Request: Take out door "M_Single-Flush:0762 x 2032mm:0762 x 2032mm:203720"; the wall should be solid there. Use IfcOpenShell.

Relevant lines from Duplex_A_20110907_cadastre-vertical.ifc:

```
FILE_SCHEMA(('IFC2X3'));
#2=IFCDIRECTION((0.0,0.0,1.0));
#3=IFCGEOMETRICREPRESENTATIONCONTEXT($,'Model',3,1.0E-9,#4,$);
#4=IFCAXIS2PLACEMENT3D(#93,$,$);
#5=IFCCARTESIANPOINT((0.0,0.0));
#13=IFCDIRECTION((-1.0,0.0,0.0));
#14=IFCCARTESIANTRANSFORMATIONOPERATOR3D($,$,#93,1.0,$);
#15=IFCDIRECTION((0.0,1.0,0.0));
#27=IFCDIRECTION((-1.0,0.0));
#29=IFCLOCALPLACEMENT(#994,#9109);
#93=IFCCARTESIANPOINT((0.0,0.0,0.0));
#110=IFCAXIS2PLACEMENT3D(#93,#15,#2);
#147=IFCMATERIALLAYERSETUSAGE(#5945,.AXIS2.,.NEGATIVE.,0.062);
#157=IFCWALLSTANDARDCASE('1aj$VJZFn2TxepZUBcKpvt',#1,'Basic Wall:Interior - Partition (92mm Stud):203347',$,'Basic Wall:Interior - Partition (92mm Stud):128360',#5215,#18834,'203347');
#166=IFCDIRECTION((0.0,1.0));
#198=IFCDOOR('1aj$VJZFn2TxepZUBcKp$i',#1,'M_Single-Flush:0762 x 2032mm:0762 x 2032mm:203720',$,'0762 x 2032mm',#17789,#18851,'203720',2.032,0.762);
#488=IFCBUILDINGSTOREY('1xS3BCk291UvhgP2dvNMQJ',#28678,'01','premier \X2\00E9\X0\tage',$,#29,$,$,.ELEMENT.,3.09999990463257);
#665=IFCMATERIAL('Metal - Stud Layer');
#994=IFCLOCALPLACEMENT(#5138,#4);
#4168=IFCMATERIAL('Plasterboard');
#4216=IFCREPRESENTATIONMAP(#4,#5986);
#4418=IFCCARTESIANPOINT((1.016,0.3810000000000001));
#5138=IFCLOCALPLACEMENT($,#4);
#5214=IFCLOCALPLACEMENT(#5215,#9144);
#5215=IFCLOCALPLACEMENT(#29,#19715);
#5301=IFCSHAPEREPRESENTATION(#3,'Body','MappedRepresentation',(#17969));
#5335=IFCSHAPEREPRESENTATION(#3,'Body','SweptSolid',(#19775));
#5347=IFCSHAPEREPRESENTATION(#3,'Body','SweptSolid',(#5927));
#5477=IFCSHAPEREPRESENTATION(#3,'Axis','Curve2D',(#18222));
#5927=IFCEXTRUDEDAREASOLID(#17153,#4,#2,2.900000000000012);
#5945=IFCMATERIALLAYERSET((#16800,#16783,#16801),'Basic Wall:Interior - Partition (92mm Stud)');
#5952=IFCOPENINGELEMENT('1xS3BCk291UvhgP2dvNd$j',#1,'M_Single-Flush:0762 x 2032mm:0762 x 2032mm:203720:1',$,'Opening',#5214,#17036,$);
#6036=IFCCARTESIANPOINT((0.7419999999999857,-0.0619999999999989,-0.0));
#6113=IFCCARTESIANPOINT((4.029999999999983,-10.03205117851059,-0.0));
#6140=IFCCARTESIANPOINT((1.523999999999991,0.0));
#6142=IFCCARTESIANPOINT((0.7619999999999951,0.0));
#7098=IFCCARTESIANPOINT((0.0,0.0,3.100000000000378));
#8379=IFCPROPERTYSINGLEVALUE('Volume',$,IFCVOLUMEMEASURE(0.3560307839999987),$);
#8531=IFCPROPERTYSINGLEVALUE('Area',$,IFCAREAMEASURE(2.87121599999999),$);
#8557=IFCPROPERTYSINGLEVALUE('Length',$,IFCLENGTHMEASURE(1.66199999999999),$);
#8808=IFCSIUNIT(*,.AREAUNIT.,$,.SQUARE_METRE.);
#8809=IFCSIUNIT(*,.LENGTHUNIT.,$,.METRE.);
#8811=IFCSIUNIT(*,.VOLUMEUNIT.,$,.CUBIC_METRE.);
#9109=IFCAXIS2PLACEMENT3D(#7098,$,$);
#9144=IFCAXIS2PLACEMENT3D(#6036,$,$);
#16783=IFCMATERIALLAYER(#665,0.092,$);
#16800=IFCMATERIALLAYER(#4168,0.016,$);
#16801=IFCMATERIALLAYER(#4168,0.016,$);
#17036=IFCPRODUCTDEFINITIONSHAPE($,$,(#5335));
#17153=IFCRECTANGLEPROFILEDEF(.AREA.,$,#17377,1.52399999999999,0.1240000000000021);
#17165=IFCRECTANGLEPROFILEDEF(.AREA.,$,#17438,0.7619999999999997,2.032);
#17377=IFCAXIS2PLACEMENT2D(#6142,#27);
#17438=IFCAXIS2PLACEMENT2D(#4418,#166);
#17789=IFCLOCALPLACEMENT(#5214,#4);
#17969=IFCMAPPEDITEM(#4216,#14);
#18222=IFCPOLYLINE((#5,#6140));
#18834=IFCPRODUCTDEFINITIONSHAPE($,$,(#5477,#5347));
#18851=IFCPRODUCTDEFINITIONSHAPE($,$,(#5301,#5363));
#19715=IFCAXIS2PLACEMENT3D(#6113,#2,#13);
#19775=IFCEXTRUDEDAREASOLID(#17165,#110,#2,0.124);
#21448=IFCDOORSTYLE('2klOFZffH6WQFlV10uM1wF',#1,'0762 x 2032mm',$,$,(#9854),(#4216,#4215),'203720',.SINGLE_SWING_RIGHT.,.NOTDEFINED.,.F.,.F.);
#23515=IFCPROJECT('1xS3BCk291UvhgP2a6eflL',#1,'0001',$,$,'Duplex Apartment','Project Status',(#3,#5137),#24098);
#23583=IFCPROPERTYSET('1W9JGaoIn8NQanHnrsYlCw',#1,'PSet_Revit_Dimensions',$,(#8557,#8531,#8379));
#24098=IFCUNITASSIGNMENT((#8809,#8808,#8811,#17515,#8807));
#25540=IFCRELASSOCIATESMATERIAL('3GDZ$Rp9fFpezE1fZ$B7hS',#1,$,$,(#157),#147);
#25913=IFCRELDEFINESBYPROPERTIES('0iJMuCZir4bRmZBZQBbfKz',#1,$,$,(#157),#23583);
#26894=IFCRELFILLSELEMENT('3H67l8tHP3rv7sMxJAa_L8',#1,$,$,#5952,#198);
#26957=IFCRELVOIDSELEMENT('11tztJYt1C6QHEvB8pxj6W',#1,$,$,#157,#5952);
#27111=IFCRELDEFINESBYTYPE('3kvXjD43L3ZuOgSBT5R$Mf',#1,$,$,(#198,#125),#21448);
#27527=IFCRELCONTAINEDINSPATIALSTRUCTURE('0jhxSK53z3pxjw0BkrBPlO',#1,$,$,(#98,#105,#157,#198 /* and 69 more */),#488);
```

```python
import ifcopenshell
import ifcopenshell.api.feature
import ifcopenshell.api.pset
import ifcopenshell.api.root
import ifcopenshell.geom
import ifcopenshell.util.element
import ifcopenshell.util.shape
import ifcopenshell.util.unit

model = ifcopenshell.open("Duplex_A_20110907_cadastre-vertical.ifc")
area_scale = ifcopenshell.util.unit.calculate_unit_scale(model, "AREAUNIT")
volume_scale = ifcopenshell.util.unit.calculate_unit_scale(model, "VOLUMEUNIT")
settings = ifcopenshell.geom.settings()


def volume(element):
    """Net volume in cubic metres, openings subtracted."""
    shape = ifcopenshell.geom.create_shape(settings, element)
    return ifcopenshell.util.shape.get_volume(shape.geometry)


door = model.by_id(198)
opening = door.FillsVoids[0].RelatingOpeningElement
wall = opening.VoidsElements[0].RelatingBuildingElement
before = volume(wall)

ifcopenshell.api.root.remove_product(model, product=door)
ifcopenshell.api.feature.remove_feature(model, feature=opening)

after = volume(wall)
thickness = 0.124  # wall thickness in metres

# Update the wall's stored quantities.
pset = model.by_id(ifcopenshell.util.element.get_pset(wall, "PSet_Revit_Dimensions", should_inherit=False)["id"])
ifcopenshell.api.pset.edit_pset(model, pset=pset, properties={
    "Area": model.create_entity("IfcAreaMeasure", after / thickness / area_scale),
    "Volume": model.create_entity("IfcVolumeMeasure", after / volume_scale),
})

print(f"wall volume {before:.3f} -> {after:.3f} m3")

model.write("Duplex_A_20110907_cadastre-vertical-out.ifc")
```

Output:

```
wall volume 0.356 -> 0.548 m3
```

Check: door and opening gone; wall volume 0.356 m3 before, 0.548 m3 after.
